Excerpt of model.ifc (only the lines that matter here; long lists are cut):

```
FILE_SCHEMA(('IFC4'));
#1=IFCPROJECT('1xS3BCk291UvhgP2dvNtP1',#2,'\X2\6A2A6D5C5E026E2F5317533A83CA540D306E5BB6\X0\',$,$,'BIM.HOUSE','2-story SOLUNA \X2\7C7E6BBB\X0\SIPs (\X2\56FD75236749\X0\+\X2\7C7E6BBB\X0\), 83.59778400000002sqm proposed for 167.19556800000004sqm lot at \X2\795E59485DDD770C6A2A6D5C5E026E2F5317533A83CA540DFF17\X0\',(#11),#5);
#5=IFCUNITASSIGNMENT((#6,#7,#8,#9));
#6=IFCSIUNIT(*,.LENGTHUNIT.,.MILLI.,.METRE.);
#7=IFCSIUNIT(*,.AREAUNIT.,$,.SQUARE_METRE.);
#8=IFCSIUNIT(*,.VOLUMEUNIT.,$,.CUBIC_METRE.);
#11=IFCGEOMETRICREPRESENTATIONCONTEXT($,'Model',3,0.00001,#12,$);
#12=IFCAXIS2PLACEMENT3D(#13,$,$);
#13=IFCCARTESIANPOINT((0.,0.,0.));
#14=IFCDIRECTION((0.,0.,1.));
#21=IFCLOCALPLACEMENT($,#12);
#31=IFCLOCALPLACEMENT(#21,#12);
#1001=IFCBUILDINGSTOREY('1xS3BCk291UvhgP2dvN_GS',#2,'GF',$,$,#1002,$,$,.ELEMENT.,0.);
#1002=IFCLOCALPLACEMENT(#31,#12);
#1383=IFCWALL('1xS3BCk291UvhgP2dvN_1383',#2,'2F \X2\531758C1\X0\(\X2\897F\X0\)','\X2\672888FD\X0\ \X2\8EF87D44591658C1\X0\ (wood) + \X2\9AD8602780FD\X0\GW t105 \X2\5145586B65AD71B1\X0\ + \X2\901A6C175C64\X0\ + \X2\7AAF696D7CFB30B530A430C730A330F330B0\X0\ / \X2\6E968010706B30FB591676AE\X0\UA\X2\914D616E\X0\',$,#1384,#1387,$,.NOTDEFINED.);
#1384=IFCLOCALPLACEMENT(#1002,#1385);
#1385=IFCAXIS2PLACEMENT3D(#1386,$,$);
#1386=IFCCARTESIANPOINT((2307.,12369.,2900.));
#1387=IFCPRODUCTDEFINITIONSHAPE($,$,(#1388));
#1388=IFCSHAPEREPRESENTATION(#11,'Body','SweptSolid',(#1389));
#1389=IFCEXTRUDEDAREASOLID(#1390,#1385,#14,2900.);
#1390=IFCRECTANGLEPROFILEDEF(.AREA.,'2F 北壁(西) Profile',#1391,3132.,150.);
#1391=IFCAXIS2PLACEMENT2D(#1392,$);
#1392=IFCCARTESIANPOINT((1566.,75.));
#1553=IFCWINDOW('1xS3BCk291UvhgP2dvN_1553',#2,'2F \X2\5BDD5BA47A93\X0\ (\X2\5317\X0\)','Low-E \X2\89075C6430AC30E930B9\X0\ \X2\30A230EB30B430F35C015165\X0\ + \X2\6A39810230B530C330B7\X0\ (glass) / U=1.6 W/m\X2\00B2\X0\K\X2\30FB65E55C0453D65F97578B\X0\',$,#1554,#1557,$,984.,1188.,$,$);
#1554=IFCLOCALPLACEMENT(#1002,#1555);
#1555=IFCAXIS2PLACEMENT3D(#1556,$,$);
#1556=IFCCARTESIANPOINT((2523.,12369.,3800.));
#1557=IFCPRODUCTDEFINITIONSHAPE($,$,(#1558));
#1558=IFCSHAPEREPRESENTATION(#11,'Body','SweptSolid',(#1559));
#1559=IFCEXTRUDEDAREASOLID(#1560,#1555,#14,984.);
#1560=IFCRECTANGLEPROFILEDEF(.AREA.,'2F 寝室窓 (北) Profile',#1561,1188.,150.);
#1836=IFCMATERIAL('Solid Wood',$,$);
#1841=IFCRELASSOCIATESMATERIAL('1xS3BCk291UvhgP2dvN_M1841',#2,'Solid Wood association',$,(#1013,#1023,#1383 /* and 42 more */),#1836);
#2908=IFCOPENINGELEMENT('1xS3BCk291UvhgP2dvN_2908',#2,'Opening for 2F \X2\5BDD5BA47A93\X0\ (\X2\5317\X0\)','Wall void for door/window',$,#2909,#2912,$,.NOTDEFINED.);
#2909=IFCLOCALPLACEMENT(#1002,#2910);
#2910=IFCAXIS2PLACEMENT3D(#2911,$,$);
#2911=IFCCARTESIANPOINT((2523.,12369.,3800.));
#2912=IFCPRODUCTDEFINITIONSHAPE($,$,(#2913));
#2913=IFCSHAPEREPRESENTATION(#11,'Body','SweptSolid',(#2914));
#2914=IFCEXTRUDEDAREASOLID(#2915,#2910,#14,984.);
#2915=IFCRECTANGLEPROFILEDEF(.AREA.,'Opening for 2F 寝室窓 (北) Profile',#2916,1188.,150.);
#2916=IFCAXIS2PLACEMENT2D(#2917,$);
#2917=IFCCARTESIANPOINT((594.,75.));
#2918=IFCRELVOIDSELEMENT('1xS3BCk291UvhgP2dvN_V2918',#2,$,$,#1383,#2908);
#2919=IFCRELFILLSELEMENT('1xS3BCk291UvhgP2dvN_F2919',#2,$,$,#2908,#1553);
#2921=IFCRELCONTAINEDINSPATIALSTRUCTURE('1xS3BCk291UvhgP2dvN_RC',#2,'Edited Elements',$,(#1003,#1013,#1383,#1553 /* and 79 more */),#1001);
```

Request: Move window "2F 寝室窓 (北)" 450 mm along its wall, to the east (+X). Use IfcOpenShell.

```python
import ifcopenshell
import ifcopenshell.api.geometry
import ifcopenshell.util.placement
import ifcopenshell.util.unit

model = ifcopenshell.open("model.ifc")
unit_scale = ifcopenshell.util.unit.calculate_unit_scale(model)

window = model.by_guid("1xS3BCk291UvhgP2dvN_1553")
opening = window.FillsVoids[0].RelatingOpeningElement
wall = opening.VoidsElements[0].RelatingBuildingElement

wall_matrix = ifcopenshell.util.placement.get_local_placement(wall.ObjectPlacement)
shift = wall_matrix[:3, 0] * 0.45 / unit_scale
before = ifcopenshell.util.placement.get_local_placement(window.ObjectPlacement)[:3, 3].copy()

# The window is not placed relative to its opening, so move both.
for product in (opening, window):
    matrix = ifcopenshell.util.placement.get_local_placement(product.ObjectPlacement)
    matrix[:3, 3] += shift
    ifcopenshell.api.geometry.edit_object_placement(model, product=product, matrix=matrix, is_si=False)

after = ifcopenshell.util.placement.get_local_placement(window.ObjectPlacement)[:3, 3]
print("window moved by", (after - before).round(3) + 0.0)

model.write("model_edited.ifc")
```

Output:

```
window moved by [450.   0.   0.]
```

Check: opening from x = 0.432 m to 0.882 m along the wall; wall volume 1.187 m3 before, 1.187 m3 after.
